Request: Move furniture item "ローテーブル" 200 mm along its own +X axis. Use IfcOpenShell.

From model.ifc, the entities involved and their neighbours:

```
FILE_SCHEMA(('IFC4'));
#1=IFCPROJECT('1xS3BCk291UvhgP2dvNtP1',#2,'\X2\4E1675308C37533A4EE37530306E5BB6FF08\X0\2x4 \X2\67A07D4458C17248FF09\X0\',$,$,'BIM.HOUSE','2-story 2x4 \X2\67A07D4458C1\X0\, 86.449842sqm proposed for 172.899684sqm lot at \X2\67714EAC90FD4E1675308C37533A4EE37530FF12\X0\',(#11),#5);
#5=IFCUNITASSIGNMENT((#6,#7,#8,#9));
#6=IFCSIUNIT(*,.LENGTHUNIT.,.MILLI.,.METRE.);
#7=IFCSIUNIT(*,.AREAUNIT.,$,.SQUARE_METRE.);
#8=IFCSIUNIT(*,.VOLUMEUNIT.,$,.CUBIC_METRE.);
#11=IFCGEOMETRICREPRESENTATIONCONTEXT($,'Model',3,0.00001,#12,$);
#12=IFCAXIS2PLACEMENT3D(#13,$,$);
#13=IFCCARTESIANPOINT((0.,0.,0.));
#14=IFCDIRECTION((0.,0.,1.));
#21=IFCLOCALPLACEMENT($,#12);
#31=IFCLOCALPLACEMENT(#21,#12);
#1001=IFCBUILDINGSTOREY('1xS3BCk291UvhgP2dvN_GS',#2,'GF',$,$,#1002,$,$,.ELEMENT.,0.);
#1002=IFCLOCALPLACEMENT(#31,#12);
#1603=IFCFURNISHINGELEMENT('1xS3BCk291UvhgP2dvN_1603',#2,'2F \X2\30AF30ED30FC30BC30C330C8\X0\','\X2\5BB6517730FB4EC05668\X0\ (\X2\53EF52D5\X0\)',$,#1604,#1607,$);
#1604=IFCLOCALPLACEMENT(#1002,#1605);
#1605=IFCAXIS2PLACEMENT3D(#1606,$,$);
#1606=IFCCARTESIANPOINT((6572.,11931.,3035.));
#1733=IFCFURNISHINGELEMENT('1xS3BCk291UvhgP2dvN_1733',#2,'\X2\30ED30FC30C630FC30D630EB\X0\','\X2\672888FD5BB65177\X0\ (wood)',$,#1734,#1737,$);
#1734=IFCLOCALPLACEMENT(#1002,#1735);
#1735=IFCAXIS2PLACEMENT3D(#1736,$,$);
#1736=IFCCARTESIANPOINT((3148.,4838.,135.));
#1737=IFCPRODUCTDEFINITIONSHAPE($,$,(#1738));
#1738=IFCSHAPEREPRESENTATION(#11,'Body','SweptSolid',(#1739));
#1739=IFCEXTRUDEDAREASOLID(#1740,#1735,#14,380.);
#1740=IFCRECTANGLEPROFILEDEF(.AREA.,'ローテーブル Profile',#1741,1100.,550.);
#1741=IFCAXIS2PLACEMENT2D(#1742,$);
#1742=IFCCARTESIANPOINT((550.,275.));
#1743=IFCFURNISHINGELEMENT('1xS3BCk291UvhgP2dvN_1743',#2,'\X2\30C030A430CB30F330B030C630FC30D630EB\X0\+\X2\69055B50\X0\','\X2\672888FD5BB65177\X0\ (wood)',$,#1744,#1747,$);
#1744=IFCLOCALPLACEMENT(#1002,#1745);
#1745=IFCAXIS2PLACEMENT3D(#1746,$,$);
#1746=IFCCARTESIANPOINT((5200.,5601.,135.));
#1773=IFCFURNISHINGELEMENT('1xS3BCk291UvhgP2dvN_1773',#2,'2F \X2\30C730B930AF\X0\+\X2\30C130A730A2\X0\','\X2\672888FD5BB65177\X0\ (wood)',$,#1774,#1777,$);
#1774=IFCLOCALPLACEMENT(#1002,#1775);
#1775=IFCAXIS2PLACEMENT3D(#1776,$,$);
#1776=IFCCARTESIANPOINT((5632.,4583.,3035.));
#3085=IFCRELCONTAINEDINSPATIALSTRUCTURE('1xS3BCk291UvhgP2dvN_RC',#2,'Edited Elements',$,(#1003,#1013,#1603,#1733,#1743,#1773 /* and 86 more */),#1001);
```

```python
import ifcopenshell
import ifcopenshell.api.geometry
import ifcopenshell.util.placement

model = ifcopenshell.open("model.ifc")

item = model.by_guid("1xS3BCk291UvhgP2dvN_1733")
matrix = ifcopenshell.util.placement.get_local_placement(item.ObjectPlacement)
matrix[:3, 3] += matrix[:3, 0] * 200.0
ifcopenshell.api.geometry.edit_object_placement(model, product=item, matrix=matrix, is_si=False)

print(ifcopenshell.util.placement.get_local_placement(item.ObjectPlacement).round(3) + 0.0)

model.write("model_rev.ifc")
```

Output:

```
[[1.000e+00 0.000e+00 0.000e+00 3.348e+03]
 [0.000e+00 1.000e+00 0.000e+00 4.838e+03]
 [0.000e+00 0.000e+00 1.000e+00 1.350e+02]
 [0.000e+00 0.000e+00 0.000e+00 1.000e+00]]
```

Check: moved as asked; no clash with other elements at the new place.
